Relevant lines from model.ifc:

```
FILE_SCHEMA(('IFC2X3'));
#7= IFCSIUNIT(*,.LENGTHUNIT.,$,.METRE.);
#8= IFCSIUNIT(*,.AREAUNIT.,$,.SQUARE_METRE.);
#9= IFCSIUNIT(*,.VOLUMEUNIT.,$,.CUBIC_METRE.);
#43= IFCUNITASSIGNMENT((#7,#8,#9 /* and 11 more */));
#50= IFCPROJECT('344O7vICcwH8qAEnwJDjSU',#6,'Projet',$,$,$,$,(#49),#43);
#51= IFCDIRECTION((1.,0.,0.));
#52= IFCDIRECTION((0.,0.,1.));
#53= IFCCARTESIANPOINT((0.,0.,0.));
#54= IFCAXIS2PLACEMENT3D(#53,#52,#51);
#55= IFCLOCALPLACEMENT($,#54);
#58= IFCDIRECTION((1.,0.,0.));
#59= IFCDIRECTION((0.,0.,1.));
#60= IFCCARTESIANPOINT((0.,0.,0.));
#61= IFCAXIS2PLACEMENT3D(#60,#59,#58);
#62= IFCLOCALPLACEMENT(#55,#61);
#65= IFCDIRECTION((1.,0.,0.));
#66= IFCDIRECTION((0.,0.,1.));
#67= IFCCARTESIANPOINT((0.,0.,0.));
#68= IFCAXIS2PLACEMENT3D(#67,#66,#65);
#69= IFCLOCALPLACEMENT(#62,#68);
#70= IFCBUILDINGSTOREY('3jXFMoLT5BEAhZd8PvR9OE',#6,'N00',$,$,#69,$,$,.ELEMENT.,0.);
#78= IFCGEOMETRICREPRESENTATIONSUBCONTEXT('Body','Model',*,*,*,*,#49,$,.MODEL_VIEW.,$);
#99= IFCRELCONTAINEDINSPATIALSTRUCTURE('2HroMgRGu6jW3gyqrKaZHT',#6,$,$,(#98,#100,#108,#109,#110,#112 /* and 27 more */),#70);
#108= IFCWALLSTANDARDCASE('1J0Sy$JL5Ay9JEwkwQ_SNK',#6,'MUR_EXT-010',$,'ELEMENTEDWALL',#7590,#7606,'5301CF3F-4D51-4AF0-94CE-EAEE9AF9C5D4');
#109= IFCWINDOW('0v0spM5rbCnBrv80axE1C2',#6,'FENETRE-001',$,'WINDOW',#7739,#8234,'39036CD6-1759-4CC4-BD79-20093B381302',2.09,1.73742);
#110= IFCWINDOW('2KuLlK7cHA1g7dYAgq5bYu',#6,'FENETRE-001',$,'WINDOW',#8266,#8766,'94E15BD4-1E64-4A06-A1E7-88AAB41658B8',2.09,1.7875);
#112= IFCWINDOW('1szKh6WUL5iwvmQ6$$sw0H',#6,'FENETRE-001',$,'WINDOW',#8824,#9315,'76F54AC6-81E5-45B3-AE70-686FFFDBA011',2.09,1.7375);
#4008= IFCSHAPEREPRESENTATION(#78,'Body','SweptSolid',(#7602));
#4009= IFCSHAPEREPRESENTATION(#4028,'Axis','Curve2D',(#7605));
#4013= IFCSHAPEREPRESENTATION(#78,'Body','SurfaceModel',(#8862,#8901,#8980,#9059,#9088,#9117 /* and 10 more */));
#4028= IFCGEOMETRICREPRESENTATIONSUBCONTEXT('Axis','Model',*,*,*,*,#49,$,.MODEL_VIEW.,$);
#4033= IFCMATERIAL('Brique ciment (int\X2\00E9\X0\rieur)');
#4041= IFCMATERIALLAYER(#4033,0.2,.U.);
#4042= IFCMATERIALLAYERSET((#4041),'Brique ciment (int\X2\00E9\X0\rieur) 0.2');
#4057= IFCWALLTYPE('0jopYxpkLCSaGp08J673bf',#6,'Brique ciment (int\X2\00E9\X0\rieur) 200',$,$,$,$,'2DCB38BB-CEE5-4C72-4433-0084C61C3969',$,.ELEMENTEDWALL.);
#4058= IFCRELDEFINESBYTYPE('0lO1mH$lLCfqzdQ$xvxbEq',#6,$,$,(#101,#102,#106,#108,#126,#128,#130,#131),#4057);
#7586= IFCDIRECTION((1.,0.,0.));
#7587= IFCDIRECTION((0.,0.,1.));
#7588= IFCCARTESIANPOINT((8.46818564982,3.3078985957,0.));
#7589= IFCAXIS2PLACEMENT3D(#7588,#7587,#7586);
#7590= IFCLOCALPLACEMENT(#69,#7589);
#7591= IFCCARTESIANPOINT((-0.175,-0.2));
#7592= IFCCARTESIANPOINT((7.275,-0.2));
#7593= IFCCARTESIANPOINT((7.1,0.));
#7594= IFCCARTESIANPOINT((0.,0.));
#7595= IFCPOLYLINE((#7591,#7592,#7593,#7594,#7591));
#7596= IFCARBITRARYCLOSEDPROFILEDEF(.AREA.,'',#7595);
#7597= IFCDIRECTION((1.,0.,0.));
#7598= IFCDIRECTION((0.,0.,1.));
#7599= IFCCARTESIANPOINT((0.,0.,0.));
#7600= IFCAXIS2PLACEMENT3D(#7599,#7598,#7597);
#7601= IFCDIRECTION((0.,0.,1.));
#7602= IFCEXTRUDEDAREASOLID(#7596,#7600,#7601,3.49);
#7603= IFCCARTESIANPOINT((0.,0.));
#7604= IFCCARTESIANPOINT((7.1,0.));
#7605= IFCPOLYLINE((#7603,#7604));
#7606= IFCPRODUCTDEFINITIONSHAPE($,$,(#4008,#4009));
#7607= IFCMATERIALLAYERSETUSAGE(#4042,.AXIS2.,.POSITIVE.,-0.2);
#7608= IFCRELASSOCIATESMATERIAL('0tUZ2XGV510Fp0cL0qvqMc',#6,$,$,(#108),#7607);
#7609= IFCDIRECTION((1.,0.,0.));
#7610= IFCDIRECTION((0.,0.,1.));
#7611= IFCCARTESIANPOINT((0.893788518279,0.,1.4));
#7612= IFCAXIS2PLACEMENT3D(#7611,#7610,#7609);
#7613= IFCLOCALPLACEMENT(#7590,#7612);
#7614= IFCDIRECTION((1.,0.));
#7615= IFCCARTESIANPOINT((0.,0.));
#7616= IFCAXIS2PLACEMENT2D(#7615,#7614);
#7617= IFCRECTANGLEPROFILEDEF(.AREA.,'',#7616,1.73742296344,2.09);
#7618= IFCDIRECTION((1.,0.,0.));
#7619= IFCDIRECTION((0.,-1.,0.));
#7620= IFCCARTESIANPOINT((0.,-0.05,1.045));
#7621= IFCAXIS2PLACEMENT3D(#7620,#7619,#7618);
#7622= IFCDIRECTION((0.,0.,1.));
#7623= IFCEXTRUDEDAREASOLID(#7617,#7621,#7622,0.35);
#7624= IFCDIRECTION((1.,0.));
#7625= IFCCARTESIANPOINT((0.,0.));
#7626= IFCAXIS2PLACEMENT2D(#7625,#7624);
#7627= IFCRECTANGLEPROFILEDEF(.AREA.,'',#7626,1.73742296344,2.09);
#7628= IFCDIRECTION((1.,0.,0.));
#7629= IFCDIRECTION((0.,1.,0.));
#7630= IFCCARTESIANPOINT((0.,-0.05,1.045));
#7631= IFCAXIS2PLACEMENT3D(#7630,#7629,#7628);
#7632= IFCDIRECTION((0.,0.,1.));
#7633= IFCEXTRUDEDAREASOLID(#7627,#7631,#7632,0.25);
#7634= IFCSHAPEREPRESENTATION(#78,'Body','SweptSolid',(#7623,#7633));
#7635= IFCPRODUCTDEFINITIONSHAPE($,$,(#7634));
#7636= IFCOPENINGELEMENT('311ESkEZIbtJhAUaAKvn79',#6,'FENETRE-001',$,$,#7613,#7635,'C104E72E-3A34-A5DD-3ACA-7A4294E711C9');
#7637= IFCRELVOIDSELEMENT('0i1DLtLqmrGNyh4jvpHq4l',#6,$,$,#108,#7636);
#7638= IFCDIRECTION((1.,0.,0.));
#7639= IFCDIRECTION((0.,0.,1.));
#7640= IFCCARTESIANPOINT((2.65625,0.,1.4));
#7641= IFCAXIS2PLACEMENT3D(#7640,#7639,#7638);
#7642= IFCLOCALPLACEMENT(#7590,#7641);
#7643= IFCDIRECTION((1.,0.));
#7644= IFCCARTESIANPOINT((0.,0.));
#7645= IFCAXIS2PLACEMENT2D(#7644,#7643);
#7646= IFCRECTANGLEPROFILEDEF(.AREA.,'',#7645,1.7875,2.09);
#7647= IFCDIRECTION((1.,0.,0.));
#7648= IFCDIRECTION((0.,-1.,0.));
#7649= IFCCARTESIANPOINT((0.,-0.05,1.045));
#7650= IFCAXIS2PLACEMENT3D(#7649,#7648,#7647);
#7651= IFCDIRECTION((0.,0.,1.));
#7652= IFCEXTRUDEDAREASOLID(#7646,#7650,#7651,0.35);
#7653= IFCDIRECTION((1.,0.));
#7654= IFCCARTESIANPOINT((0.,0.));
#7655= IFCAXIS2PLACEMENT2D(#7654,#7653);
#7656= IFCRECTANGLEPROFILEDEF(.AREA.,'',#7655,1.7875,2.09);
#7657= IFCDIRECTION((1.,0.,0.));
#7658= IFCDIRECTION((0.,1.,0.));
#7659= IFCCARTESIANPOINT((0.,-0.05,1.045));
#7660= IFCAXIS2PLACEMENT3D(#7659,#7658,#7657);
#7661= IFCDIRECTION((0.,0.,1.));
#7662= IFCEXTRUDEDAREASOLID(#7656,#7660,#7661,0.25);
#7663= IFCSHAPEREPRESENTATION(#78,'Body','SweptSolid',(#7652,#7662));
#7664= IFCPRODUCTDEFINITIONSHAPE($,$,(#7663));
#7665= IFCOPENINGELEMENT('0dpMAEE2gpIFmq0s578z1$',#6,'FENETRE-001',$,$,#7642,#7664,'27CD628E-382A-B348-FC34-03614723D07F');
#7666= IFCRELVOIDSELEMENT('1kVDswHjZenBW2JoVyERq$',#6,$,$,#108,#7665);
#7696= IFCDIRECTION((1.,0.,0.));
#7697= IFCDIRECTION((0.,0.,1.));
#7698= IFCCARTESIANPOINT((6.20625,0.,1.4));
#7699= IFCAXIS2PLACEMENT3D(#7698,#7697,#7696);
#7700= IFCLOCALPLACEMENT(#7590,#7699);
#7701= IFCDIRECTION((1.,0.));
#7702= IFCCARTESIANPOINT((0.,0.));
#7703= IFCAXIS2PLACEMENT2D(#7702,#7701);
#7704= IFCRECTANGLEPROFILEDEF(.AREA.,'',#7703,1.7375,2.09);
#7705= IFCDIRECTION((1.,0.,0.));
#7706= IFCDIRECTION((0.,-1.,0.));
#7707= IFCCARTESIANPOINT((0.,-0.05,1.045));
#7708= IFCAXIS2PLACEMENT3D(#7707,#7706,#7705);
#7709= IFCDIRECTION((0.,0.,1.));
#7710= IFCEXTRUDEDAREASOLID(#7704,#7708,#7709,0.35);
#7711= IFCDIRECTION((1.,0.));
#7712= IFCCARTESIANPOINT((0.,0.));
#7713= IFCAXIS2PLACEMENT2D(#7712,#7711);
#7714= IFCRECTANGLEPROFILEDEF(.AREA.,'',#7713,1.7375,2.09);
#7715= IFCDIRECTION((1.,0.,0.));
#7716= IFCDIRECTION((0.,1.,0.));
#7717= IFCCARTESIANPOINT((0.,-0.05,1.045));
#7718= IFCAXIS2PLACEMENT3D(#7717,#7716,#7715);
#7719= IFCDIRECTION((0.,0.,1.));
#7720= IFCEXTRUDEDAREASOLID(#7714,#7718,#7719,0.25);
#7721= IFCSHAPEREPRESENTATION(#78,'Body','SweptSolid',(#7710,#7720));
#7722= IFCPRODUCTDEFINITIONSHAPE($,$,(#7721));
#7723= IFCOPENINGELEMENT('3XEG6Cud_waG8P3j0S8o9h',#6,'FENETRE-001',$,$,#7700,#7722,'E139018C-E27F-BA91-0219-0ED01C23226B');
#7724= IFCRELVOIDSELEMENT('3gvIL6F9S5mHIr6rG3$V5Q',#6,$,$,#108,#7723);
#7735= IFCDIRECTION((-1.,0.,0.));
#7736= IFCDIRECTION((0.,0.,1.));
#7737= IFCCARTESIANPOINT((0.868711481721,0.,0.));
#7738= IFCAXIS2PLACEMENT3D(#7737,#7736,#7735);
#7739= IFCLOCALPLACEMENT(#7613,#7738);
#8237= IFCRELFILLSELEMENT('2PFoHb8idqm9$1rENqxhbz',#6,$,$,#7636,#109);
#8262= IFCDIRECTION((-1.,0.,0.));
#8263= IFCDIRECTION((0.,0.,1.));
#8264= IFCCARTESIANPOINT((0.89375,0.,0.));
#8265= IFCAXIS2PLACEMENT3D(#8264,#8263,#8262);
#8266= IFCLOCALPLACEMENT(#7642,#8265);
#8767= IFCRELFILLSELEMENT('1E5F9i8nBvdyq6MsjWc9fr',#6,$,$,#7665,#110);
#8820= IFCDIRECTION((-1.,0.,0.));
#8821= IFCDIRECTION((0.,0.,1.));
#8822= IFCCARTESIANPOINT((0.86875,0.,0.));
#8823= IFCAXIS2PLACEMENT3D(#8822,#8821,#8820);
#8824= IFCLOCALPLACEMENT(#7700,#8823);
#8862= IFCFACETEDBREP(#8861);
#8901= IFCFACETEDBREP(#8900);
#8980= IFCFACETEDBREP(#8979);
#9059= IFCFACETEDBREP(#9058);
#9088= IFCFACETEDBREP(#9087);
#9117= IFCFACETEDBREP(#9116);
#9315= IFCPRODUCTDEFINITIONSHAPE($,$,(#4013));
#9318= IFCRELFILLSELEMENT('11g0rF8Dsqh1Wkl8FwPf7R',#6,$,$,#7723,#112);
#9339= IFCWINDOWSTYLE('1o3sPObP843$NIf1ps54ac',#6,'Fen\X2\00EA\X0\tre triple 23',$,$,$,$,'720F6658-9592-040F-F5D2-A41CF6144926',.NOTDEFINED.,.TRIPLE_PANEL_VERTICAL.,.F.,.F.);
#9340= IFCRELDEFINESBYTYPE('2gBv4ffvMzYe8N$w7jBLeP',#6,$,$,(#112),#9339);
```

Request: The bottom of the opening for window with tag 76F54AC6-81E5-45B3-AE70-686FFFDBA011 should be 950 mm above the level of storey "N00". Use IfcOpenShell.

```python
import numpy as np
import ifcopenshell
import ifcopenshell.api.geometry
import ifcopenshell.geom
import ifcopenshell.util.element
import ifcopenshell.util.placement
import ifcopenshell.util.shape
import ifcopenshell.util.unit

model = ifcopenshell.open("model.ifc")
unit_scale = ifcopenshell.util.unit.calculate_unit_scale(model)

window = model.by_guid("1szKh6WUL5iwvmQ6$$sw0H")
opening = window.FillsVoids[0].RelatingOpeningElement
storey = ifcopenshell.util.element.get_container(window, ifc_class="IfcBuildingStorey")
level = ifcopenshell.util.placement.get_local_placement(storey.ObjectPlacement)[2, 3]

# The opening's origin need not be at the sill, so measure its lowest point.
shape = ifcopenshell.geom.create_shape(ifcopenshell.geom.settings(), opening)
bottom = ifcopenshell.util.shape.get_shape_bottom_elevation(shape, shape.geometry) / unit_scale
dz = level + 0.95 / unit_scale - bottom

shift = np.array([0.0, 0.0, dz])
# The window is placed relative to its opening, so it follows when the opening moves.
matrix = ifcopenshell.util.placement.get_local_placement(opening.ObjectPlacement)
matrix[:3, 3] += shift
ifcopenshell.api.geometry.edit_object_placement(
    model, product=opening, matrix=matrix, is_si=False, should_transform_children=True
)

print(f"moved by {dz * unit_scale:+.3f} m")

model.write("model_rev.ifc")
```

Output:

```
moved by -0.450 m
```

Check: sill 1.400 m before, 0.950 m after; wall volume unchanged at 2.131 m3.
